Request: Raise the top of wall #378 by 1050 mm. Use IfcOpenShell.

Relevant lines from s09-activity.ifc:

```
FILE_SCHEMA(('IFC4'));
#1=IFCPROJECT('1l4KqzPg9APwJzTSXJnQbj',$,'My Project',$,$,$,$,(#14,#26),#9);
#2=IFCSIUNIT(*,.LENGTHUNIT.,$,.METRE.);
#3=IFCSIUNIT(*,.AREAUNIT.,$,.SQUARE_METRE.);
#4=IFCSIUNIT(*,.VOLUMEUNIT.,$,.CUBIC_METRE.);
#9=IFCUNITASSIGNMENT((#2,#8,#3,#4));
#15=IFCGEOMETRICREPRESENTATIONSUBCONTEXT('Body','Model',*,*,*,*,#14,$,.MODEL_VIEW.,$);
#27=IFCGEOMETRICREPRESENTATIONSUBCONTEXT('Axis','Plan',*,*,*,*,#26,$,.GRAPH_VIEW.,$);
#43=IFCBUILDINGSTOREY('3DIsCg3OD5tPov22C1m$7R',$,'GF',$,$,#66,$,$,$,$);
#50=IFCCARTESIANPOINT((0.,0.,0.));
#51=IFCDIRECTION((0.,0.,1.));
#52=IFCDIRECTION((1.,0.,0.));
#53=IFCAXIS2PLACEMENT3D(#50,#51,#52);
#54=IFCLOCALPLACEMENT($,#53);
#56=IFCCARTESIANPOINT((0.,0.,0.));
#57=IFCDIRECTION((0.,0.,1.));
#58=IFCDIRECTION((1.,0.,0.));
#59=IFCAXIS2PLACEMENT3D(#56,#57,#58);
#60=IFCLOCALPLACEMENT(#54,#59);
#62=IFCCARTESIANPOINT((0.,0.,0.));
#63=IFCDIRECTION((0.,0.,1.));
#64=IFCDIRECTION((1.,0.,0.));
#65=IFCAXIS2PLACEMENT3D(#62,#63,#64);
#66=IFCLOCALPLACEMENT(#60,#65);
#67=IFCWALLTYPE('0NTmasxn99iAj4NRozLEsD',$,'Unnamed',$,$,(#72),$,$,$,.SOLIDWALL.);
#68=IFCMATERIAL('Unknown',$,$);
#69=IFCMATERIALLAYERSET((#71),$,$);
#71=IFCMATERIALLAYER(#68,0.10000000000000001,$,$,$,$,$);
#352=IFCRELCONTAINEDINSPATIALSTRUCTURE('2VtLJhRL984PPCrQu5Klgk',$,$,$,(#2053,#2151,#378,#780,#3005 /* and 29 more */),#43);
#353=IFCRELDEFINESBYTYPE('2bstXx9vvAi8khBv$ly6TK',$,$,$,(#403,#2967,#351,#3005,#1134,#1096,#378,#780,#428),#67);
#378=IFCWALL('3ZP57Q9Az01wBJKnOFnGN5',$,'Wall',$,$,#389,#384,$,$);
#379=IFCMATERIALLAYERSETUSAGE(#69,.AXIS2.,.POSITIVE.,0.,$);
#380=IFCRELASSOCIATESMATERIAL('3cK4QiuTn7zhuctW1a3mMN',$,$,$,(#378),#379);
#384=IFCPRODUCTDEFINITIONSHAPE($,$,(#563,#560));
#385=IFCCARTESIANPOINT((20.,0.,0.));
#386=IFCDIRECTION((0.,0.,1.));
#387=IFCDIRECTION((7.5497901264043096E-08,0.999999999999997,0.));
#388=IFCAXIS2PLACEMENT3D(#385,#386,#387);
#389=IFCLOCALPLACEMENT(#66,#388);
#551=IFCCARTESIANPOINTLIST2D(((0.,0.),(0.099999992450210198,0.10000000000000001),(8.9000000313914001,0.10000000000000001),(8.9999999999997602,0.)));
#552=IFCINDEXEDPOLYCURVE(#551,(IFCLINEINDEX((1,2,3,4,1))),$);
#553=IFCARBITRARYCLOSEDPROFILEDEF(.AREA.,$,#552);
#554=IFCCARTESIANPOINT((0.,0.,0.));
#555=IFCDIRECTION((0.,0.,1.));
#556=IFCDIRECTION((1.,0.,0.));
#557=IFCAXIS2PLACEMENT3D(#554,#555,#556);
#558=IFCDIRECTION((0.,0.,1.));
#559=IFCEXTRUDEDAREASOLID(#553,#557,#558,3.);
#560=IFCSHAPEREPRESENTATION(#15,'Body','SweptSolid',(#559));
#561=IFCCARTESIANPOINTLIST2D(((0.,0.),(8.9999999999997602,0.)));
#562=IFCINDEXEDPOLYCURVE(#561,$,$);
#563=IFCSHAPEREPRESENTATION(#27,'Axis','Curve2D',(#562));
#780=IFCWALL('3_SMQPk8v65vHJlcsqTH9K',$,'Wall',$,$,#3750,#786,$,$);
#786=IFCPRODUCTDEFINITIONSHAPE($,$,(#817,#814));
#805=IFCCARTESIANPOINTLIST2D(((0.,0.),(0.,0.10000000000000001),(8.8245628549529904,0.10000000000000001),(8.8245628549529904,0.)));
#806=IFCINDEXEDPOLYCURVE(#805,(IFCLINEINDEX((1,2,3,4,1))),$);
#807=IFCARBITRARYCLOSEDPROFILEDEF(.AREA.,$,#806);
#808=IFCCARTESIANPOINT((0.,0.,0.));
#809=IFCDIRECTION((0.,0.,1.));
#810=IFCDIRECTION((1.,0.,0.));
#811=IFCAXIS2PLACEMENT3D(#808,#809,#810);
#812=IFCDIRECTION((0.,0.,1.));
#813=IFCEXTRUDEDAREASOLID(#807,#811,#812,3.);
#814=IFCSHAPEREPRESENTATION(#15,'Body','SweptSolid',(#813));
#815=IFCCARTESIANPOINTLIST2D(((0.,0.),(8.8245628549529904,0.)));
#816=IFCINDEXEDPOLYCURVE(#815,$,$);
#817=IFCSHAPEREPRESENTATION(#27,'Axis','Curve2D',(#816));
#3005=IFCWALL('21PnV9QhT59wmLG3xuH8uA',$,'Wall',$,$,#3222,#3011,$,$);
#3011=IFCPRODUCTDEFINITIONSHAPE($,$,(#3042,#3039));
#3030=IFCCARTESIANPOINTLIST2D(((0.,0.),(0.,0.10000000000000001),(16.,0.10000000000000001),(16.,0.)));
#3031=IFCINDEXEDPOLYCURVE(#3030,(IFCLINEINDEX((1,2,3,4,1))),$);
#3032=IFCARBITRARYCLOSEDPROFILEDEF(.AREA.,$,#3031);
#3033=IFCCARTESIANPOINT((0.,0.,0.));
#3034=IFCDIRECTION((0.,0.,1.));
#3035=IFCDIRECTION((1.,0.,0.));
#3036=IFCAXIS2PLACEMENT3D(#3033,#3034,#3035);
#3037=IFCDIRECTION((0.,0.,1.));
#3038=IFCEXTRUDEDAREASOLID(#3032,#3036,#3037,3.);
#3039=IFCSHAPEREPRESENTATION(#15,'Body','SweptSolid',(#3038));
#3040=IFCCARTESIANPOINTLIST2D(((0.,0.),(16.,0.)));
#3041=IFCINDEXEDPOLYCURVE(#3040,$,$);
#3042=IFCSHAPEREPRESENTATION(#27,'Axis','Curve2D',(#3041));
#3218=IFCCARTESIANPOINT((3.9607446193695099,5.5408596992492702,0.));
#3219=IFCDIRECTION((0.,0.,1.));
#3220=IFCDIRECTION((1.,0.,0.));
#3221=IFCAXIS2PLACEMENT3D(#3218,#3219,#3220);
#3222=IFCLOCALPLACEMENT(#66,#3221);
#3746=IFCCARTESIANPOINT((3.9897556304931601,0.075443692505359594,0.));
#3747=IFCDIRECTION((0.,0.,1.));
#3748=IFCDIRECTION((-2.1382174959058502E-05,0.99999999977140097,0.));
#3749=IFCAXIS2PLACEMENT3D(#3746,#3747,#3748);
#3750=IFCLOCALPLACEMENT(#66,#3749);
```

```python
import ifcopenshell
import ifcopenshell.geom
import ifcopenshell.util.representation
import ifcopenshell.util.shape
import ifcopenshell.util.unit

model = ifcopenshell.open("s09-activity.ifc")
unit_scale = ifcopenshell.util.unit.calculate_unit_scale(model)
settings = ifcopenshell.geom.settings()


def volume(element):
    """Net volume in cubic metres, openings subtracted."""
    shape = ifcopenshell.geom.create_shape(settings, element)
    return ifcopenshell.util.shape.get_volume(shape.geometry)


wall = model.by_id(378)
before = volume(wall)

body = ifcopenshell.util.representation.get_representation(wall, "Model", "Body")
solid = body.Items[0]
old_height = solid.Depth
solid.Depth += 1.05 / unit_scale
after = volume(wall)

print(f"height {old_height:g} -> {solid.Depth:g}, volume {before:.3f} -> {after:.3f} m3")

model.write("s09-activity_rev.ifc")
```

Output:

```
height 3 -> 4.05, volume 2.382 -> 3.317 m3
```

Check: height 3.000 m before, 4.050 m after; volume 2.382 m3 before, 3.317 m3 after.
